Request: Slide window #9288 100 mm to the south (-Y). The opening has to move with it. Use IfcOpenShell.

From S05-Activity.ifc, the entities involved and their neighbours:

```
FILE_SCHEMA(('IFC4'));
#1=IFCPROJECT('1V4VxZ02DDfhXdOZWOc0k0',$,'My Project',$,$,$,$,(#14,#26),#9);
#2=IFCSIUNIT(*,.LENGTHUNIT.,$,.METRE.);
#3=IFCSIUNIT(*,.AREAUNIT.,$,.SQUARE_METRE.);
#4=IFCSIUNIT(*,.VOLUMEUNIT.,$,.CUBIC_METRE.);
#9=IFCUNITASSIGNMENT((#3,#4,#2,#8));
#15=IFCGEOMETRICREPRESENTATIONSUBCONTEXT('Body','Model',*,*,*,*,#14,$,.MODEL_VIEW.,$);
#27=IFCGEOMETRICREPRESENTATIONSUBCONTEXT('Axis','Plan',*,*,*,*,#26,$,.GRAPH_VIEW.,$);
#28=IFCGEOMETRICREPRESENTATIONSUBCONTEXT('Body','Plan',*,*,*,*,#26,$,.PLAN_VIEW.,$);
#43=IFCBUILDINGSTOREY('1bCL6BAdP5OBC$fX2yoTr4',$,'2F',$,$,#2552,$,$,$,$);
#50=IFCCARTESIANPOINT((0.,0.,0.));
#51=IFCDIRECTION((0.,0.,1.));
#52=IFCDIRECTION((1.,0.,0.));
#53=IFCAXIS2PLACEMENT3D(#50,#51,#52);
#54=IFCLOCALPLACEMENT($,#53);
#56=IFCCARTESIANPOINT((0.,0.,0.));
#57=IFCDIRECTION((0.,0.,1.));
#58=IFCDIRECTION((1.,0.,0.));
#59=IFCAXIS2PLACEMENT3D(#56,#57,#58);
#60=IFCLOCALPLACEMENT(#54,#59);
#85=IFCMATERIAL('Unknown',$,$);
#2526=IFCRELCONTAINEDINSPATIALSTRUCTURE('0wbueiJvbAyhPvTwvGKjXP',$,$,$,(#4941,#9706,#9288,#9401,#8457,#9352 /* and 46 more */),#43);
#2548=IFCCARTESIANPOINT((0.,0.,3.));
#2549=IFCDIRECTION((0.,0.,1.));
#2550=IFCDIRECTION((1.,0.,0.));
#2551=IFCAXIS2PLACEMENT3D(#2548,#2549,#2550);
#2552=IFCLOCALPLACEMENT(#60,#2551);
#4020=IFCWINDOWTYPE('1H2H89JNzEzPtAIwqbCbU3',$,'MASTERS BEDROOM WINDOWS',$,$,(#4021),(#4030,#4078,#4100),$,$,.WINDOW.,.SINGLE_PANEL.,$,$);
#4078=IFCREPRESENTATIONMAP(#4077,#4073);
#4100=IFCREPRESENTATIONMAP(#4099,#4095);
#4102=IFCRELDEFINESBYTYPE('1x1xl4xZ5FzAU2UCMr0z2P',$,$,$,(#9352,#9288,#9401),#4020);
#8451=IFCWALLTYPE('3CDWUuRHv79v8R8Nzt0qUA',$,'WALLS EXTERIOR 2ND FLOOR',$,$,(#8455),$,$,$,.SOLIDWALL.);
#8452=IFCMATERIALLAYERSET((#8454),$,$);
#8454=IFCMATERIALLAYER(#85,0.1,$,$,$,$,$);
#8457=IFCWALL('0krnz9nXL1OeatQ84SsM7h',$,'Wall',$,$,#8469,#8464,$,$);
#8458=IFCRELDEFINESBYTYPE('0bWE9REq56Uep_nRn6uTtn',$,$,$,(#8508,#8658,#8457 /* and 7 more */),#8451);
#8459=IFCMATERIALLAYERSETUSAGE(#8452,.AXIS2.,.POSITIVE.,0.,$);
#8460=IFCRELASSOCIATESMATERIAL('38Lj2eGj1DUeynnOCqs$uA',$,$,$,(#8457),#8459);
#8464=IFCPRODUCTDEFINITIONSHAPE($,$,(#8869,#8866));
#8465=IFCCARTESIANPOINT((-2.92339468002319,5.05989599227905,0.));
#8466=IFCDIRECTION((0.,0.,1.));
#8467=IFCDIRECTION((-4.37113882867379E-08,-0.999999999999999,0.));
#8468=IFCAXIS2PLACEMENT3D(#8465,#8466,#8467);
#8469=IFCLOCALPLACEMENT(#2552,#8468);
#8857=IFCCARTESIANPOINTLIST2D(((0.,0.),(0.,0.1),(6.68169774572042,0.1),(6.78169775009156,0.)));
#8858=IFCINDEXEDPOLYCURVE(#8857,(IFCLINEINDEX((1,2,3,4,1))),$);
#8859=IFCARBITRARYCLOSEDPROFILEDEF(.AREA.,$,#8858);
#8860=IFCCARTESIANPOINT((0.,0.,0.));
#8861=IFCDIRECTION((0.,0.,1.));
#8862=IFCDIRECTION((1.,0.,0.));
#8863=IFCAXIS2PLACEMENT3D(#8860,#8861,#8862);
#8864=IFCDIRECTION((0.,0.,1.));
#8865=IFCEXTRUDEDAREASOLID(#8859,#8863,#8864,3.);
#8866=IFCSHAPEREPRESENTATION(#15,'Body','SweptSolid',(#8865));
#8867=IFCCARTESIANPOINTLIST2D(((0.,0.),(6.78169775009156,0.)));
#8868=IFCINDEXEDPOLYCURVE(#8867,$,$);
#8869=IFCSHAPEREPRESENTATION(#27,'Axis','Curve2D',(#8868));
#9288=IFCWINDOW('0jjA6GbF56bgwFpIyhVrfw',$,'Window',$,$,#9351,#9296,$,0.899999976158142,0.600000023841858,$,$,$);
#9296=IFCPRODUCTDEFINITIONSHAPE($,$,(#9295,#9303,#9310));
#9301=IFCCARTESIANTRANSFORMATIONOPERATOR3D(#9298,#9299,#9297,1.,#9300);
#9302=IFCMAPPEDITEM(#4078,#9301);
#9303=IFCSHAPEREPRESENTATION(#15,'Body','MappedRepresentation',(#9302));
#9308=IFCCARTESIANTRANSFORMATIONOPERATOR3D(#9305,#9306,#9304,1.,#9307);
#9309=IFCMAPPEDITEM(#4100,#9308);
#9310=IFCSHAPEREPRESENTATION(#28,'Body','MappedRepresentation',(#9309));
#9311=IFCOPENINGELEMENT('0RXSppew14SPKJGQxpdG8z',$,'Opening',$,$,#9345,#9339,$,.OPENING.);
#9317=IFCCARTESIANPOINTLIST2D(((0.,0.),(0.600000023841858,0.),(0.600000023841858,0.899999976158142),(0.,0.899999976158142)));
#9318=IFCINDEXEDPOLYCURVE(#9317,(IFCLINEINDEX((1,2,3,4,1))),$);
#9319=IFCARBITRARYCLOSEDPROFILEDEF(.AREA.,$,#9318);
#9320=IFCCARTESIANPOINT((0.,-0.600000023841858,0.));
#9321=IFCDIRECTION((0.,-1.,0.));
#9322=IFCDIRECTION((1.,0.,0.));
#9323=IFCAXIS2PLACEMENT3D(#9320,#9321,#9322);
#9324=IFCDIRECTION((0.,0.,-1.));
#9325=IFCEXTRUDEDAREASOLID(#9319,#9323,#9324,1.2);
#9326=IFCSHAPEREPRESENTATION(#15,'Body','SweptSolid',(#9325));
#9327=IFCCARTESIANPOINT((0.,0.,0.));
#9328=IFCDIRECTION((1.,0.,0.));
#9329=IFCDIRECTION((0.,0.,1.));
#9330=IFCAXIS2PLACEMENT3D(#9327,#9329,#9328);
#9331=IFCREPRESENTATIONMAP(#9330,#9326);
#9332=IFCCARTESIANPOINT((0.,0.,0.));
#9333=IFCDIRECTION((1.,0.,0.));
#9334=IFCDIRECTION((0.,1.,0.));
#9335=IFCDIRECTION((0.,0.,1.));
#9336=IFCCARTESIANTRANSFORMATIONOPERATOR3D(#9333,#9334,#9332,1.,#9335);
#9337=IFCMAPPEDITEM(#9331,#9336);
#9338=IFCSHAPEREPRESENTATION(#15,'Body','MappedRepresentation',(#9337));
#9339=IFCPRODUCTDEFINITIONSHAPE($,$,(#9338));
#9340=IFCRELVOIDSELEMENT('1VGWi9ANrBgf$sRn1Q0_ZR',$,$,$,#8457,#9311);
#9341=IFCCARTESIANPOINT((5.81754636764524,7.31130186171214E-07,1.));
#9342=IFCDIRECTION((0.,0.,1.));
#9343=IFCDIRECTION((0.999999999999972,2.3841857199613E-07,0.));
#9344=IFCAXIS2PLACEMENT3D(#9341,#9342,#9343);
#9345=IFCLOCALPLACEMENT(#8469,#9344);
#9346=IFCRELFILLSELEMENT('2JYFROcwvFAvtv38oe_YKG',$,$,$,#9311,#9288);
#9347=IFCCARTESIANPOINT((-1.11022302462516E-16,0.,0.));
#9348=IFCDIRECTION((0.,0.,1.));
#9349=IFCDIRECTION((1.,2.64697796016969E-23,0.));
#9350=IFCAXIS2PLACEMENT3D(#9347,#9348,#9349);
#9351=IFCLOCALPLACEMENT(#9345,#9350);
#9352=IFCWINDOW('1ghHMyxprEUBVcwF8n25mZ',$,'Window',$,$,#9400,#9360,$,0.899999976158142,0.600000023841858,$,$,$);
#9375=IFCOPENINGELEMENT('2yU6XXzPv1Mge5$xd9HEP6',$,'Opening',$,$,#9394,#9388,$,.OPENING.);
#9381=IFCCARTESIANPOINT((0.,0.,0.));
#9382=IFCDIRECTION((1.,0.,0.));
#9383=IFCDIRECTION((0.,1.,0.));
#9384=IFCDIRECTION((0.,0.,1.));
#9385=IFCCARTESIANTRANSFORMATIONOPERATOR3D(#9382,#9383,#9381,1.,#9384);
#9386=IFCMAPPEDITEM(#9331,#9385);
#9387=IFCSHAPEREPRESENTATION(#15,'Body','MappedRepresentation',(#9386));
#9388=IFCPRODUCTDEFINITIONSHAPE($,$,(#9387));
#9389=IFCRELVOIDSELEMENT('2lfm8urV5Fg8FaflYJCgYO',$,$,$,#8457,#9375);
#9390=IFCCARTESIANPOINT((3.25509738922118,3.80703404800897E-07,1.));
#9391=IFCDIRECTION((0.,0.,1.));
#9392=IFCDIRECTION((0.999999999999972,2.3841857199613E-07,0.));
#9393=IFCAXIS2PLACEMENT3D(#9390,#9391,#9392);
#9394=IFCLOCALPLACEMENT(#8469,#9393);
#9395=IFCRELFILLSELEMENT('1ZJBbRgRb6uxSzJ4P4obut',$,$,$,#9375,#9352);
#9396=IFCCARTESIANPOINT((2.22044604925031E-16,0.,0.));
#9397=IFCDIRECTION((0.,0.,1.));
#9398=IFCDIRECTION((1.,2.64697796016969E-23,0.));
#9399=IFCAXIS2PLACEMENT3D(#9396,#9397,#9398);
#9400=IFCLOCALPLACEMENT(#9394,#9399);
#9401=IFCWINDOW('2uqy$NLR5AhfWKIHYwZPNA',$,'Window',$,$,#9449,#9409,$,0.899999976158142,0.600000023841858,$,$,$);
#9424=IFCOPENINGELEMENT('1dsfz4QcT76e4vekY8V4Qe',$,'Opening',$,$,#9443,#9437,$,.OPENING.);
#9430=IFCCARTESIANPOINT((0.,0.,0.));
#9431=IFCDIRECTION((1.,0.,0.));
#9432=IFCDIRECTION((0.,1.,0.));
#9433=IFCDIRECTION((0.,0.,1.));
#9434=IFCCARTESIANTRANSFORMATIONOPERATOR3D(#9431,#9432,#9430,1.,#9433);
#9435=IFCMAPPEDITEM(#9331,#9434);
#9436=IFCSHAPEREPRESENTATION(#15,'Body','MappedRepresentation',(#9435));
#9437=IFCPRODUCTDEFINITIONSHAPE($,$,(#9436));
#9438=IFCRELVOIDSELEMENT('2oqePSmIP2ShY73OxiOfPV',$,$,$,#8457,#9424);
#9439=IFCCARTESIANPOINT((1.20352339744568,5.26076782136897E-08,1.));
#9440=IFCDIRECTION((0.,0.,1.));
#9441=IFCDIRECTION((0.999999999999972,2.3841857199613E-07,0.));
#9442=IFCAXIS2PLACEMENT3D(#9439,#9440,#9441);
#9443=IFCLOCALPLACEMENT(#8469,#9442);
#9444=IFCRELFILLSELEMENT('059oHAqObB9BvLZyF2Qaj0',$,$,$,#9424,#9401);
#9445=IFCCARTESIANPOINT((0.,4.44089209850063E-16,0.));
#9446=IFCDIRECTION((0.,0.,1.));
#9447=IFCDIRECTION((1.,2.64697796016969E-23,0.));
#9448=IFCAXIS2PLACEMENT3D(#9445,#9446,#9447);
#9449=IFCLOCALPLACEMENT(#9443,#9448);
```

```python
import ifcopenshell
import ifcopenshell.api.geometry
import ifcopenshell.util.placement
import ifcopenshell.util.unit

model = ifcopenshell.open("S05-Activity.ifc")
unit_scale = ifcopenshell.util.unit.calculate_unit_scale(model)

window = model.by_guid("0jjA6GbF56bgwFpIyhVrfw")
opening = window.FillsVoids[0].RelatingOpeningElement
wall = opening.VoidsElements[0].RelatingBuildingElement

wall_matrix = ifcopenshell.util.placement.get_local_placement(wall.ObjectPlacement)
shift = wall_matrix[:3, 0] * 0.1 / unit_scale
before = ifcopenshell.util.placement.get_local_placement(window.ObjectPlacement)[:3, 3].copy()

# The window is placed relative to its opening, so it follows when the opening moves.
matrix = ifcopenshell.util.placement.get_local_placement(opening.ObjectPlacement)
matrix[:3, 3] += shift
ifcopenshell.api.geometry.edit_object_placement(
    model, product=opening, matrix=matrix, is_si=False, should_transform_children=True
)

after = ifcopenshell.util.placement.get_local_placement(window.ObjectPlacement)[:3, 3]
print("window moved by", (after - before).round(3) + 0.0)

model.write("S05-Activity_edited.ifc")
```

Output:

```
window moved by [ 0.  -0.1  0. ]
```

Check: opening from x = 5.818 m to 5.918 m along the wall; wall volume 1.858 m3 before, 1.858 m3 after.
